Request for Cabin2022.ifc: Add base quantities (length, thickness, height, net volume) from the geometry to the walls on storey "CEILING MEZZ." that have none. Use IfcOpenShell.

First a look at what the model holds.

```python
import ifcopenshell
import ifcopenshell.util.element
import ifcopenshell.util.unit

model = ifcopenshell.open("Cabin2022.ifc")
print(model.schema)
for unit_type in ("LENGTHUNIT", "AREAUNIT", "VOLUMEUNIT"):
    print(unit_type, ifcopenshell.util.unit.calculate_unit_scale(model, unit_type))
storey = next(s for s in model.by_type("IfcBuildingStorey") if s.Name == "CEILING MEZZ.")
walls = [e for e in ifcopenshell.util.element.get_decomposition(storey) if e.is_a("IfcWall")]
for e in sorted(walls, key=lambda e: e.id()):
    print(e.id(), e.is_a(), e.Name, list(ifcopenshell.util.element.get_psets(e, qtos_only=True)), sep=" | ")
```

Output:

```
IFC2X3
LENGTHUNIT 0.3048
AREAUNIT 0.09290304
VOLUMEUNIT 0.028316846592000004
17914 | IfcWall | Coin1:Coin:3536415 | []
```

```python
import ifcopenshell
import ifcopenshell.api.pset
import ifcopenshell.geom
import ifcopenshell.util.element
import ifcopenshell.util.shape
import ifcopenshell.util.unit

model = ifcopenshell.open("Cabin2022.ifc")
unit_scale = ifcopenshell.util.unit.calculate_unit_scale(model)
volume_scale = ifcopenshell.util.unit.calculate_unit_scale(model, "VOLUMEUNIT")
settings = ifcopenshell.geom.settings()

storey = next(s for s in model.by_type("IfcBuildingStorey") if s.Name == "CEILING MEZZ.")
walls = [e for e in ifcopenshell.util.element.get_decomposition(storey) if e.is_a("IfcWall")]

for e in sorted(walls, key=lambda e: e.id()):
    if ifcopenshell.util.element.get_psets(e, qtos_only=True, should_inherit=False):
        continue
    # Geometry comes back in metres, in the element's own axes.
    shape = ifcopenshell.geom.create_shape(settings, e)
    values = {
        "Length": ifcopenshell.util.shape.get_x(shape.geometry) / unit_scale,
        "Width": ifcopenshell.util.shape.get_y(shape.geometry) / unit_scale,
        "Height": ifcopenshell.util.shape.get_z(shape.geometry) / unit_scale,
        "NetVolume": ifcopenshell.util.shape.get_volume(shape.geometry) / volume_scale,
    }
    qto = ifcopenshell.api.pset.add_qto(model, product=e, name="BaseQuantities")
    ifcopenshell.api.pset.edit_qto(model, qto=qto, properties=values)
    print(e.id(), {k: round(v, 3) for k, v in values.items()})

model.write("Cabin2022_rev.ifc")
```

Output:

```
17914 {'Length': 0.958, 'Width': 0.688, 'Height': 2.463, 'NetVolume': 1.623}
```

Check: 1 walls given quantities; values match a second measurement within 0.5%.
